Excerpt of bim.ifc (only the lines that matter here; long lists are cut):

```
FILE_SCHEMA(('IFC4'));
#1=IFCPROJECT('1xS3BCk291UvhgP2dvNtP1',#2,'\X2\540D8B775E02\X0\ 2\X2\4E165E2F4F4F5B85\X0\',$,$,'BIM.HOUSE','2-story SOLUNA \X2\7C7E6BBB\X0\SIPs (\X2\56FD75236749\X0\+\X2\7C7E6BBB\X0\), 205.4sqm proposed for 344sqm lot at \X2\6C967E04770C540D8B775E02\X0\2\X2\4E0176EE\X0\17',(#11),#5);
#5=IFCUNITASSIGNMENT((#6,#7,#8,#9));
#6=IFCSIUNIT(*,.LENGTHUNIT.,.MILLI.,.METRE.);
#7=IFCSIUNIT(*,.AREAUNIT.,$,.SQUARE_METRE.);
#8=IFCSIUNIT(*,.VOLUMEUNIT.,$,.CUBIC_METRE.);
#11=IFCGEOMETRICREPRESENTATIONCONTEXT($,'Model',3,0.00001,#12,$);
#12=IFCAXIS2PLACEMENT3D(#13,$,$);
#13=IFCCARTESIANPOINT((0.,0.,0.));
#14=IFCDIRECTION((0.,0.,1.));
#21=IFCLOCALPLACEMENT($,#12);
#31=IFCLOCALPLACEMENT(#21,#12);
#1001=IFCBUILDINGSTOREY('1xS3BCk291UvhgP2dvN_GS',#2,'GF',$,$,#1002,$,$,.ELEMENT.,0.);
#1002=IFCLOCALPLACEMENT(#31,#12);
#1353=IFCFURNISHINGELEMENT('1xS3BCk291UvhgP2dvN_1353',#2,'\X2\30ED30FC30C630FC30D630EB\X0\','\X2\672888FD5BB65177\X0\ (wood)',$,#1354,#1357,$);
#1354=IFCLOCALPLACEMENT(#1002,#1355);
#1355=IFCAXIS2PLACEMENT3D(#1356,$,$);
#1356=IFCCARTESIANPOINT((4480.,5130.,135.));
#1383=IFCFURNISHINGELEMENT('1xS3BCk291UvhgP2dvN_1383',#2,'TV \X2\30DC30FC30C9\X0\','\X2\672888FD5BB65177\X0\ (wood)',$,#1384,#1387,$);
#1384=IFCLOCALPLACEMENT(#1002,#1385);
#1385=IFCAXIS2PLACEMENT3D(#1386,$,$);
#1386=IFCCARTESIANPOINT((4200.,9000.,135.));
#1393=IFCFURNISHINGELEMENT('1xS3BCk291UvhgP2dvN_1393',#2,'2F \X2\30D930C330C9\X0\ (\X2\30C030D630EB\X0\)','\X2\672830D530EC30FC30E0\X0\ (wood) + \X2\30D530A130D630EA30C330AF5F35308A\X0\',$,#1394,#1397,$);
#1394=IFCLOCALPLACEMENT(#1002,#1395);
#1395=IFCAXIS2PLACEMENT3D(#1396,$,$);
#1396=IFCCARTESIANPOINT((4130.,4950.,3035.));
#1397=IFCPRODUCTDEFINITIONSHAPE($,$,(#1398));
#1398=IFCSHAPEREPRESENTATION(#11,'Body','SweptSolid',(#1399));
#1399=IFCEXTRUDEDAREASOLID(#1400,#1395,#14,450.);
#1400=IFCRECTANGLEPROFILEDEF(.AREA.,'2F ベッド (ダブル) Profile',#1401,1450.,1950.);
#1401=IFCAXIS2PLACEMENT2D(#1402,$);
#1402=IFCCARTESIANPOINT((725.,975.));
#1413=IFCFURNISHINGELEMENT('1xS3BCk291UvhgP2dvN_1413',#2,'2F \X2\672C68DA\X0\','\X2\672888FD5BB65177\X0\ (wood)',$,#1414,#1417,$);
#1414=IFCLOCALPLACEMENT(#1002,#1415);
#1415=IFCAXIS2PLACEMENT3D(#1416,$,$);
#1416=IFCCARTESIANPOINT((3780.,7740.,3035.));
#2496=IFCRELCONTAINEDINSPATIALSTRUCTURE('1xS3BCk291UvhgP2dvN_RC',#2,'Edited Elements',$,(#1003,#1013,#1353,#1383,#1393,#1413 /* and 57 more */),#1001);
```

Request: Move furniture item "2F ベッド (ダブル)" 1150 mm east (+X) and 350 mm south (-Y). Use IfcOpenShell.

```python
import ifcopenshell
import ifcopenshell.api.geometry
import ifcopenshell.util.placement
import ifcopenshell.util.unit

model = ifcopenshell.open("bim.ifc")
unit_scale = ifcopenshell.util.unit.calculate_unit_scale(model)

item = model.by_guid("1xS3BCk291UvhgP2dvN_1393")
matrix = ifcopenshell.util.placement.get_local_placement(item.ObjectPlacement)
matrix[0, 3] += 1.15 / unit_scale
matrix[1, 3] -= 0.35 / unit_scale
ifcopenshell.api.geometry.edit_object_placement(model, product=item, matrix=matrix, is_si=False)

print(ifcopenshell.util.placement.get_local_placement(item.ObjectPlacement).round(3) + 0.0)

model.write("bim_v2.ifc")
```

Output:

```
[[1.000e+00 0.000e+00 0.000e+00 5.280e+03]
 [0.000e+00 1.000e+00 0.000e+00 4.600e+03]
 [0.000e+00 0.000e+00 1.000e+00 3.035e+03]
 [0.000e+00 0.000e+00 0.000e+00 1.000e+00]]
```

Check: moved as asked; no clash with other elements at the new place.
